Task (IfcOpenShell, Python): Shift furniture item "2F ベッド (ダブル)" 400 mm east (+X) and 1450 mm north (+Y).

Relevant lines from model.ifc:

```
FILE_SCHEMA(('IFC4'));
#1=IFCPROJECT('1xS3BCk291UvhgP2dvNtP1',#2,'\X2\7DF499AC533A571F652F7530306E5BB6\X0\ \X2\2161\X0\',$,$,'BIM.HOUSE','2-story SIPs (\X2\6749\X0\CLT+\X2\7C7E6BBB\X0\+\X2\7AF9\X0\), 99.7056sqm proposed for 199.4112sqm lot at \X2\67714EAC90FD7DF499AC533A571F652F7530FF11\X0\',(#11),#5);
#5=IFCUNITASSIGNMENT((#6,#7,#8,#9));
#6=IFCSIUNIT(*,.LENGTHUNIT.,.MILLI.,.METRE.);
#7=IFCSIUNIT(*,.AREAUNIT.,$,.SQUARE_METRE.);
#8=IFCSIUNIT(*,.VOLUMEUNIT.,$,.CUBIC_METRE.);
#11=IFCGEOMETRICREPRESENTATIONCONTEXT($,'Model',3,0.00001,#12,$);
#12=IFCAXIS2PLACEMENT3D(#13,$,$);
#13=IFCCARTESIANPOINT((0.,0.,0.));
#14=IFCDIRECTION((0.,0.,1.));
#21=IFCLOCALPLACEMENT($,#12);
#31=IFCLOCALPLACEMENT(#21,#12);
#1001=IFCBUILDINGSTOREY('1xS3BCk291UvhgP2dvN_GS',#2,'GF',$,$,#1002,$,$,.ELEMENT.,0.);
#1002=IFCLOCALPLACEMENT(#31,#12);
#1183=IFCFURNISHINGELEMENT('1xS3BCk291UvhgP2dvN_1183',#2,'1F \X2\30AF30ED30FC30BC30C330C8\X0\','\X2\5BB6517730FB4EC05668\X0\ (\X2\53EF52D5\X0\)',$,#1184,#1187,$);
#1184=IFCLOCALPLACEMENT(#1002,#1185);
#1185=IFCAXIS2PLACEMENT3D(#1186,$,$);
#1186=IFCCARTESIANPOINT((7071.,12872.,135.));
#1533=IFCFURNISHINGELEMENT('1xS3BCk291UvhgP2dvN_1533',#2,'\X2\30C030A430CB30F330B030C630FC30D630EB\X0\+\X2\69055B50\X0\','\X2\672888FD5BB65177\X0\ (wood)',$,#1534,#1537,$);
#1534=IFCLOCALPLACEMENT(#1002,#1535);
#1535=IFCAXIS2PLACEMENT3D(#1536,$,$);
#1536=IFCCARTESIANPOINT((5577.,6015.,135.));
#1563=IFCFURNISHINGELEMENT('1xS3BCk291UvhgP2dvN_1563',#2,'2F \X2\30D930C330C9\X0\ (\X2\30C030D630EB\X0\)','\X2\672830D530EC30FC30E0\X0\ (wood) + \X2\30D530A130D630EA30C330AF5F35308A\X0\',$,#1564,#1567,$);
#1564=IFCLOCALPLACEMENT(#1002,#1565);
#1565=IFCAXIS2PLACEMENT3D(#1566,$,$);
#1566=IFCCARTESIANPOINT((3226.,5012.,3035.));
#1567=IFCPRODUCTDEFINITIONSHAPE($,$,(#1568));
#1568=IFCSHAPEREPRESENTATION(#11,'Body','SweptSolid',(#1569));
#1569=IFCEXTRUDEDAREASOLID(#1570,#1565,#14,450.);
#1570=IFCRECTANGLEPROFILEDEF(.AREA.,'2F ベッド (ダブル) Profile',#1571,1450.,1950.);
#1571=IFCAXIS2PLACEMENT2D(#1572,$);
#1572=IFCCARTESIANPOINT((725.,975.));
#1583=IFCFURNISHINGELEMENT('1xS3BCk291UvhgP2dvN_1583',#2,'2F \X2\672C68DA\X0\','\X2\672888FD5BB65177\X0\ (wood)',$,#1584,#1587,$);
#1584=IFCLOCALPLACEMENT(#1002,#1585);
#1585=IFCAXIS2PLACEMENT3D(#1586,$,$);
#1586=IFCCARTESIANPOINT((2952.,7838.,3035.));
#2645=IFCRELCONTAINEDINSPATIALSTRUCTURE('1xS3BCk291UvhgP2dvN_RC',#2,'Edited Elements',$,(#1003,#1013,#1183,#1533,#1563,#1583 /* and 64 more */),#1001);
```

```python
import ifcopenshell
import ifcopenshell.api.geometry
import ifcopenshell.util.placement

model = ifcopenshell.open("model.ifc")

item = model.by_guid("1xS3BCk291UvhgP2dvN_1563")
matrix = ifcopenshell.util.placement.get_local_placement(item.ObjectPlacement)
matrix[0, 3] += 400.0
matrix[1, 3] += 1450.0
ifcopenshell.api.geometry.edit_object_placement(model, product=item, matrix=matrix, is_si=False)

print(ifcopenshell.util.placement.get_local_placement(item.ObjectPlacement).round(3) + 0.0)

model.write("model_rev.ifc")
```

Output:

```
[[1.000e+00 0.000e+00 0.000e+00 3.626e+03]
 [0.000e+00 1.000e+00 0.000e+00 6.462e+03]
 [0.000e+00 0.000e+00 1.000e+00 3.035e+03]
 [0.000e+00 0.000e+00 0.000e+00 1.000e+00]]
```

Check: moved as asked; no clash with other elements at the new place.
